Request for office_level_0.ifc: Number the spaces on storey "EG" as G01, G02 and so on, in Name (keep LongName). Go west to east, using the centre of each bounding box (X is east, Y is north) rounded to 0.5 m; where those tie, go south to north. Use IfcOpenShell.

First a look at what the model holds.

```python
import ifcopenshell
import ifcopenshell.util.element
import ifcopenshell.util.placement

model = ifcopenshell.open("office_level_0.ifc")
print(model.schema)
storey = next(s for s in model.by_type("IfcBuildingStorey") if s.Name == "EG")
spaces = [e for e in ifcopenshell.util.element.get_decomposition(storey) if e.is_a("IfcSpace")]
for e in sorted(spaces, key=lambda e: e.id()):
    origin = ifcopenshell.util.placement.get_local_placement(e.ObjectPlacement)[:3, 3]
    print(e.id(), e.Name, e.LongName, origin.round(2) + 0.0, sep=" | ")
```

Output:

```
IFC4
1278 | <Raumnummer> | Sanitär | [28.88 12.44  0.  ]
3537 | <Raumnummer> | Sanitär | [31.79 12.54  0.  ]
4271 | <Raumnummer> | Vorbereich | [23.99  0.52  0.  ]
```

```python
import ifcopenshell
import ifcopenshell.geom
import ifcopenshell.util.element
import ifcopenshell.util.shape

model = ifcopenshell.open("office_level_0.ifc")
settings = ifcopenshell.geom.settings()
settings.set("use-world-coords", True)


def centre(element):
    shape = ifcopenshell.geom.create_shape(settings, element)
    return ifcopenshell.util.shape.get_bbox_centroid(shape.geometry)


storey = next(s for s in model.by_type("IfcBuildingStorey") if s.Name == "EG")
spaces = [e for e in ifcopenshell.util.element.get_decomposition(storey) if e.is_a("IfcSpace")]

# Insertion points can sit at a corner or the storey origin, so sort by the geometry (in metres).
centres = {e: centre(e) for e in spaces}
spaces.sort(key=lambda e: (round(centres[e][0] / 0.5), centres[e][1]))

for i, e in enumerate(spaces, start=1):
    number = f"G{i:02d}"
    e.Name = number
    print(e.id(), number)

model.write("office_level_0-out.ifc")
```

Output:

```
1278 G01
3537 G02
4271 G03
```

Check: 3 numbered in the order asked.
